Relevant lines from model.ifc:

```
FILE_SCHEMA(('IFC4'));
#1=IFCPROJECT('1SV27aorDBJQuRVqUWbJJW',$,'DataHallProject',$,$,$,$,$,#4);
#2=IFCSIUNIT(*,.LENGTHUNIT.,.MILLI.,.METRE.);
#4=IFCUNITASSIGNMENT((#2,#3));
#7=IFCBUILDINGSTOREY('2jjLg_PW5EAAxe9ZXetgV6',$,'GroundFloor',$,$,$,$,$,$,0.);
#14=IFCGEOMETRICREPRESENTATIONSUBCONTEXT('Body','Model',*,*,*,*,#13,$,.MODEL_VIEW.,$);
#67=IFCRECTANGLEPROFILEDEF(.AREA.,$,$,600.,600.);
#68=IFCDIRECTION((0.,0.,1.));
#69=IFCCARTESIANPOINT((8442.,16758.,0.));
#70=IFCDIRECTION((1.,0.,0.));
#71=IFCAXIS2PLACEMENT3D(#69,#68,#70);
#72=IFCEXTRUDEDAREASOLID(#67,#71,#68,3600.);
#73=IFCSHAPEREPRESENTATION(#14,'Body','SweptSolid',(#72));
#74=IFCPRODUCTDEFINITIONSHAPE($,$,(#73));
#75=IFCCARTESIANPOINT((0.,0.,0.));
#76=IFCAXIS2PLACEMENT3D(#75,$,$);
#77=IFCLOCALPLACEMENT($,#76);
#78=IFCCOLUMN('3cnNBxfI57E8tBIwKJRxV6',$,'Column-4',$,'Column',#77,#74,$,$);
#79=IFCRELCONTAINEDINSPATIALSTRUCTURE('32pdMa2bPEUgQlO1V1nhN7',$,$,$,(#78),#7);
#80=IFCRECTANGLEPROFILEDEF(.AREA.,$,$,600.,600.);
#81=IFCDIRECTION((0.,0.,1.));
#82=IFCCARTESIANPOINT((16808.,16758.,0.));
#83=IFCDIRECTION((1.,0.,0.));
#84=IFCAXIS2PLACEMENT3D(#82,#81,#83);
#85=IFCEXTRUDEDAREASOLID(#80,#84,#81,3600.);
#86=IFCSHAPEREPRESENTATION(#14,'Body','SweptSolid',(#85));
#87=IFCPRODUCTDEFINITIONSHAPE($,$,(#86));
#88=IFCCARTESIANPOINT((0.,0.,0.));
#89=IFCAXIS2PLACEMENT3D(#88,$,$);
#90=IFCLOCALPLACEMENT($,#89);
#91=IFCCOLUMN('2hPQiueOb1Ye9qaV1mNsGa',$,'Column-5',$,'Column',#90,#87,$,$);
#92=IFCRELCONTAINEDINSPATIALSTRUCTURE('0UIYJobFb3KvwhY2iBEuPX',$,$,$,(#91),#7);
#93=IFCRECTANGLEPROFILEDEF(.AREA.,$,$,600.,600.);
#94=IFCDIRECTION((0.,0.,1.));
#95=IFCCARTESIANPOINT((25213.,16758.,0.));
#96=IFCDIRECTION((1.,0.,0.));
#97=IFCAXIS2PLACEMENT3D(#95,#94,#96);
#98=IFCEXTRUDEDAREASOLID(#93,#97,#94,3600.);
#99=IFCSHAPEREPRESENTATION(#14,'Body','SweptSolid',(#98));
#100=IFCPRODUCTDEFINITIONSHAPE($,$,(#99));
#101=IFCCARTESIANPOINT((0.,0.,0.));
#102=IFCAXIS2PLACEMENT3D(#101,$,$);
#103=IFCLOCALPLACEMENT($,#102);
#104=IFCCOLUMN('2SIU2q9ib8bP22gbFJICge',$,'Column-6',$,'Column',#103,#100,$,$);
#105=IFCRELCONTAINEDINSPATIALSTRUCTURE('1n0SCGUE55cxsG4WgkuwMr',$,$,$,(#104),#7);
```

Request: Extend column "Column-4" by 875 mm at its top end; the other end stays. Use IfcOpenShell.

```python
import ifcopenshell
import ifcopenshell.util.representation

model = ifcopenshell.open("model.ifc")

member = model.by_guid("3cnNBxfI57E8tBIwKJRxV6")
change = 875.0

# The extrusion runs towards the end named, so only its depth changes.
body = ifcopenshell.util.representation.get_representation(member, "Model", "Body")
solid = body.Items[0]
old_length = solid.Depth
solid.Depth += change

print(f"length {old_length:g} -> {solid.Depth:g}")

model.write("model_v2.ifc")
```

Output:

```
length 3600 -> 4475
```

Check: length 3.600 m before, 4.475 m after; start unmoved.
